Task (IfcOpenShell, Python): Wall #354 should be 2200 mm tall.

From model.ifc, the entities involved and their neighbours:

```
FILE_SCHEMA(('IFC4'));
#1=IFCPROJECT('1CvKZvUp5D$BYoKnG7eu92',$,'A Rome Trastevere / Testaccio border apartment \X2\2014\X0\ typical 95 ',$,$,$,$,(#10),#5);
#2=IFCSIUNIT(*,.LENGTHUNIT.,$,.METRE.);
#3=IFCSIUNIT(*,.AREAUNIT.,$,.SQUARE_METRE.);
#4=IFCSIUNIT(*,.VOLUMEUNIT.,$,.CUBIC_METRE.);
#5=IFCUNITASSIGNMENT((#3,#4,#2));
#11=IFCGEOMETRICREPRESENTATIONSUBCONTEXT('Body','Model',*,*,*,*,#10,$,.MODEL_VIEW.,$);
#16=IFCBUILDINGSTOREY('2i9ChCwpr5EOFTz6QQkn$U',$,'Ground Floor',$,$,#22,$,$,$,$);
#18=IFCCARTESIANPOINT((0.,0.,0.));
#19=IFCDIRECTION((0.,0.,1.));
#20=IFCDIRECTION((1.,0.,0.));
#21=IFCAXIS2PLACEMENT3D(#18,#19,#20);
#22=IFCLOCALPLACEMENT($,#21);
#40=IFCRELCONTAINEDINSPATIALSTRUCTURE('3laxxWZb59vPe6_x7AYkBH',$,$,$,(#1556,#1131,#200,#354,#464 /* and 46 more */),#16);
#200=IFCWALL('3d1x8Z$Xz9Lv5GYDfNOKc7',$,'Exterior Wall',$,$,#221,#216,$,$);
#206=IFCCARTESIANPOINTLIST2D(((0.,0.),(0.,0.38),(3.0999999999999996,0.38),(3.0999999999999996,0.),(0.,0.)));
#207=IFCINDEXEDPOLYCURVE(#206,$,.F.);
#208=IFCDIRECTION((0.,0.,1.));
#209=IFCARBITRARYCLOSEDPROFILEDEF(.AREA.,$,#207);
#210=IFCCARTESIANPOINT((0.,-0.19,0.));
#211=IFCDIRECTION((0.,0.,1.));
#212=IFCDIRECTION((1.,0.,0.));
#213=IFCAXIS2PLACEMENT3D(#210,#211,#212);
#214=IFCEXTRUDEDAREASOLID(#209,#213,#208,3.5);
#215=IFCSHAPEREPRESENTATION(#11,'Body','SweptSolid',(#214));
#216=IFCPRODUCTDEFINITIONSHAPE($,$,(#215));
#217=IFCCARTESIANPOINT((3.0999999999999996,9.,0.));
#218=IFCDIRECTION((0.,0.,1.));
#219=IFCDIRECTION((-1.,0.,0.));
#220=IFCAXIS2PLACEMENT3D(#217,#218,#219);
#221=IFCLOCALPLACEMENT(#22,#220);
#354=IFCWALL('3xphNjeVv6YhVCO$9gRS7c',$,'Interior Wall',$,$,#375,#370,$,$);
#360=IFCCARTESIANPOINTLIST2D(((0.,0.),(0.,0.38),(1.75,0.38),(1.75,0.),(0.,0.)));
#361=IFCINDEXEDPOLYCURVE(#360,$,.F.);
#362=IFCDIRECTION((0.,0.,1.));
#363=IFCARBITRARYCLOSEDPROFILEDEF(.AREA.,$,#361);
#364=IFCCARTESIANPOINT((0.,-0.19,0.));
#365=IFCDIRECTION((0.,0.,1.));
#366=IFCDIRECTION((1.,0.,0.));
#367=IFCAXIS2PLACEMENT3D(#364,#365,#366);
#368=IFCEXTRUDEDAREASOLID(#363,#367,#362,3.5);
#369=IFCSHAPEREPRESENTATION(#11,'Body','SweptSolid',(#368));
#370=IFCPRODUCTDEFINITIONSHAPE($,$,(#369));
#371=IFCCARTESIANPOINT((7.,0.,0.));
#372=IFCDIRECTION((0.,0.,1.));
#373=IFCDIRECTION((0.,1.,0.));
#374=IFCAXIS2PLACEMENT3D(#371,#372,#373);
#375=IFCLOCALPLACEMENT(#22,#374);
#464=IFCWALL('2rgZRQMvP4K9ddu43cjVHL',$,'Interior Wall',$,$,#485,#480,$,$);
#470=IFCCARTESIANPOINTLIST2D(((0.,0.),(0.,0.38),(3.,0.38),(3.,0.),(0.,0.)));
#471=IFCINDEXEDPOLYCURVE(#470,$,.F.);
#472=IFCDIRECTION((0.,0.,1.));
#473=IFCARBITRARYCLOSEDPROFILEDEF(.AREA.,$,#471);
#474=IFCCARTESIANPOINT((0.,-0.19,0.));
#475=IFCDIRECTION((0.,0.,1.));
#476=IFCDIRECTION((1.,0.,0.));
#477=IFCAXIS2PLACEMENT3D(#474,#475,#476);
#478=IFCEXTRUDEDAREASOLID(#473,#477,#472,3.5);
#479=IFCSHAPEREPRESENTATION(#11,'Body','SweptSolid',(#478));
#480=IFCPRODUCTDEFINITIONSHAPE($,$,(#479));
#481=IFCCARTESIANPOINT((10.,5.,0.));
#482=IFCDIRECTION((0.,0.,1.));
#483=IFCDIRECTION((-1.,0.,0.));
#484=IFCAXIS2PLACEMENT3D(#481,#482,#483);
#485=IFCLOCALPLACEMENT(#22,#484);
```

```python
import ifcopenshell
import ifcopenshell.geom
import ifcopenshell.util.representation
import ifcopenshell.util.shape

model = ifcopenshell.open("model.ifc")
settings = ifcopenshell.geom.settings()


def volume(element):
    """Net volume in cubic metres, openings subtracted."""
    shape = ifcopenshell.geom.create_shape(settings, element)
    return ifcopenshell.util.shape.get_volume(shape.geometry)


wall = model.by_guid("3xphNjeVv6YhVCO$9gRS7c")
before = volume(wall)

body = ifcopenshell.util.representation.get_representation(wall, "Model", "Body")
solid = body.Items[0]
old_height = solid.Depth
solid.Depth = 2.2
after = volume(wall)

print(f"height {old_height:g} -> {solid.Depth:g}, volume {before:.3f} -> {after:.3f} m3")

model.write("model_updated.ifc")
```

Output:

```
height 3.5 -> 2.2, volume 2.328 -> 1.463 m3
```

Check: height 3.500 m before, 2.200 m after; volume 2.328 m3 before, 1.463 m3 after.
